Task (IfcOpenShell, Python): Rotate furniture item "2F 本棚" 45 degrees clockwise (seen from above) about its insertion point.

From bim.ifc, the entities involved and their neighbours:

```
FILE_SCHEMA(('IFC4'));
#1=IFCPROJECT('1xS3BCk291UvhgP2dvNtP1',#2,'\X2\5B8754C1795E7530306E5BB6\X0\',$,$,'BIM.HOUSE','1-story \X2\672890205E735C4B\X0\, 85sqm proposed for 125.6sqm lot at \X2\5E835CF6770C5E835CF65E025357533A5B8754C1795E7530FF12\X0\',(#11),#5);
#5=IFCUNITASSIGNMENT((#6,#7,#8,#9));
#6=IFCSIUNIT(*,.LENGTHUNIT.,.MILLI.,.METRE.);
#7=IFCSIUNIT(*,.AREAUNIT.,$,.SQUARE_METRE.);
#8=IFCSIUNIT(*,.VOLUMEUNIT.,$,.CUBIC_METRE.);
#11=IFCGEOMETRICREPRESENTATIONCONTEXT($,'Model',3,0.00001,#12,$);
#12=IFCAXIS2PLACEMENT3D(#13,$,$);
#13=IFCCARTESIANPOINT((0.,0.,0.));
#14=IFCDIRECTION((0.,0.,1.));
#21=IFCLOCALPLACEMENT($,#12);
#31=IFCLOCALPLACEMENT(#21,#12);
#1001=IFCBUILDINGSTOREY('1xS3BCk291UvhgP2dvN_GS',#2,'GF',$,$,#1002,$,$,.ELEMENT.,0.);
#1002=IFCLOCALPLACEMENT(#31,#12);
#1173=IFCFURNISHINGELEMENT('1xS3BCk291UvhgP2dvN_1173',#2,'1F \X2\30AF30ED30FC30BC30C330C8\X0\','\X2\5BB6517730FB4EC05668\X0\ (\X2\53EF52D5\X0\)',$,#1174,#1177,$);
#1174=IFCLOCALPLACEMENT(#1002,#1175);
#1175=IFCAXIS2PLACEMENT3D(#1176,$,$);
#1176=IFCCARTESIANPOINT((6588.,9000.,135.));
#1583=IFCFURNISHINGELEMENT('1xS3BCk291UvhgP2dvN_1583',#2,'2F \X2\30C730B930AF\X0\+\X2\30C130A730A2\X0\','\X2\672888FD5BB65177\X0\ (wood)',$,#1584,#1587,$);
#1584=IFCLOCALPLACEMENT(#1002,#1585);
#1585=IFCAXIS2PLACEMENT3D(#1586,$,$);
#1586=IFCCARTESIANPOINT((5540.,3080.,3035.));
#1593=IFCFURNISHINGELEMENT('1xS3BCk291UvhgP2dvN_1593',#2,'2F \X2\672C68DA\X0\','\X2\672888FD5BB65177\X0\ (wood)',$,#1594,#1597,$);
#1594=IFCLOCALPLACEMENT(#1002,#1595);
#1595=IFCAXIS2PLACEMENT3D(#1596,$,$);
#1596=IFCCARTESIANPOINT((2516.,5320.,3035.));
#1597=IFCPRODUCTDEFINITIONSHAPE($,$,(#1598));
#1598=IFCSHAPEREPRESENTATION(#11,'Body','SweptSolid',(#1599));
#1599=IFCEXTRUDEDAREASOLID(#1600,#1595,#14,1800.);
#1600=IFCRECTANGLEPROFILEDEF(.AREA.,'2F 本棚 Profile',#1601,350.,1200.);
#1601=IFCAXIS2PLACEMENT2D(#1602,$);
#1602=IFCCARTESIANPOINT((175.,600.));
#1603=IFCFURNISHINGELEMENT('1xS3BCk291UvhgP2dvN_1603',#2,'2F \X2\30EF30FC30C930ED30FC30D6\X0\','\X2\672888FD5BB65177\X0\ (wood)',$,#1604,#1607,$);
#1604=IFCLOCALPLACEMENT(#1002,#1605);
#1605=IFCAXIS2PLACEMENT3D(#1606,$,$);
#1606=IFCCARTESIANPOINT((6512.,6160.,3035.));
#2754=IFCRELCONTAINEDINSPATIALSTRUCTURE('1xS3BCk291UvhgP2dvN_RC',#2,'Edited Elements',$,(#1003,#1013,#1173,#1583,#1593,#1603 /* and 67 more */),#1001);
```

```python
import ifcopenshell
import ifcopenshell.api.geometry
import ifcopenshell.util.placement

model = ifcopenshell.open("bim.ifc")

item = model.by_guid("1xS3BCk291UvhgP2dvN_1593")
matrix = ifcopenshell.util.placement.get_local_placement(item.ObjectPlacement)
matrix = matrix @ ifcopenshell.util.placement.rotation(-45, "Z")
ifcopenshell.api.geometry.edit_object_placement(model, product=item, matrix=matrix, is_si=False)

print(ifcopenshell.util.placement.get_local_placement(item.ObjectPlacement).round(3) + 0.0)

model.write("bim_updated.ifc")
```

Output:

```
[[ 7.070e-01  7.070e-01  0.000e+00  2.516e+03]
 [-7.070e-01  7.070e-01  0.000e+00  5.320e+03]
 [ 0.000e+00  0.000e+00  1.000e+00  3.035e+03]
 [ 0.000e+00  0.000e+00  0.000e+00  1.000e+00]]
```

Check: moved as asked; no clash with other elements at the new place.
